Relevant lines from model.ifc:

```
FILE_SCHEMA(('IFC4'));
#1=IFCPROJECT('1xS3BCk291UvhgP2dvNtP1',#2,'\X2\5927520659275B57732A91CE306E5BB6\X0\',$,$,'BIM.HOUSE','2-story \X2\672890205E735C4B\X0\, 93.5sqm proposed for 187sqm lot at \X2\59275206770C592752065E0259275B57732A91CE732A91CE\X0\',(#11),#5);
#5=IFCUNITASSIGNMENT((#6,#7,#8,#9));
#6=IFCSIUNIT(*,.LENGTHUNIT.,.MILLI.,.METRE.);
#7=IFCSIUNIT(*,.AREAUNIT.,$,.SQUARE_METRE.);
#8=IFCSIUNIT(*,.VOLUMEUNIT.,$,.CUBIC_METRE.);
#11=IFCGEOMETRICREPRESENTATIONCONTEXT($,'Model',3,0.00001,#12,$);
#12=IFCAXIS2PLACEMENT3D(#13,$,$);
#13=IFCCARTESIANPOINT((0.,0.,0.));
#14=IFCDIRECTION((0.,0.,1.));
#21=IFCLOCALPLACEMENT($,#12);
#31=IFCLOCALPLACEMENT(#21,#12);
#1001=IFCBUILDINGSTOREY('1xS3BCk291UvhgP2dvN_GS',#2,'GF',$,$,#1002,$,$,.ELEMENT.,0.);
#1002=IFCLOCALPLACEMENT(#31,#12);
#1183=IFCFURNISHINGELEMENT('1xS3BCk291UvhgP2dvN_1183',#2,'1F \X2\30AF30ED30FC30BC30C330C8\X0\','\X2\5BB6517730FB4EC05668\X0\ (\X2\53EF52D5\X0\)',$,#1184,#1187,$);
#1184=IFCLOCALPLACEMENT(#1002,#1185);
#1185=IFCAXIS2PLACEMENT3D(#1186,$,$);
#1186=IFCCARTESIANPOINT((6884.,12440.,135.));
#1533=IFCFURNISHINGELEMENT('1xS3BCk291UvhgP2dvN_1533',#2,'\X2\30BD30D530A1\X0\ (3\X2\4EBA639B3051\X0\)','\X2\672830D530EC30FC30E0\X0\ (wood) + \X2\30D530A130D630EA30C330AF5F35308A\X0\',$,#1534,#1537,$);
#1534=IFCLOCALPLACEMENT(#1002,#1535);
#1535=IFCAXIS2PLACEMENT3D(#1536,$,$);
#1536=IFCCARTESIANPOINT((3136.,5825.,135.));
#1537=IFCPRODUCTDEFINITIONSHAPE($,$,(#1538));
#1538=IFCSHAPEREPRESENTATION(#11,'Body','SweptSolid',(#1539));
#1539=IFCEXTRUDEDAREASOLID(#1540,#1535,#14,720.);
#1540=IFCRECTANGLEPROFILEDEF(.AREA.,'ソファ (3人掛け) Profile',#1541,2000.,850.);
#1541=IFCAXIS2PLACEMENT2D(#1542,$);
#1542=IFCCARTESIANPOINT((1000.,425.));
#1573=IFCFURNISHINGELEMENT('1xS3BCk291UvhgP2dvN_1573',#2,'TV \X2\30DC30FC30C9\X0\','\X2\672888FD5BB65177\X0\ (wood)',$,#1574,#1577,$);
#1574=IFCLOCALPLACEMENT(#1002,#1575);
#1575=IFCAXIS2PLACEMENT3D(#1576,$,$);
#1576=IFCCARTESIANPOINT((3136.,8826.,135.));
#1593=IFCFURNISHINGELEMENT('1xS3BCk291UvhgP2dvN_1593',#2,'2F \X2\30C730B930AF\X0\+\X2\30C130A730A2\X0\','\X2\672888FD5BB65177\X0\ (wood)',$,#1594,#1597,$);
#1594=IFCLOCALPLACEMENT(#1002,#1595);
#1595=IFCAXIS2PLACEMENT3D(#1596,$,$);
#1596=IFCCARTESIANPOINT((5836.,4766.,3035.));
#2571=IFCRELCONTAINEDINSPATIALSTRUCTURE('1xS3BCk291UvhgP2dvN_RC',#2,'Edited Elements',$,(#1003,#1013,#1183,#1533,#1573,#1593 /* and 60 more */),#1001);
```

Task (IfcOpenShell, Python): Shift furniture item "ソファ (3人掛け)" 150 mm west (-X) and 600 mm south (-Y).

```python
import ifcopenshell
import ifcopenshell.api.geometry
import ifcopenshell.util.placement

model = ifcopenshell.open("model.ifc")

item = model.by_id(1533)
matrix = ifcopenshell.util.placement.get_local_placement(item.ObjectPlacement)
matrix[0, 3] -= 150.0
matrix[1, 3] -= 600.0
ifcopenshell.api.geometry.edit_object_placement(model, product=item, matrix=matrix, is_si=False)

print(ifcopenshell.util.placement.get_local_placement(item.ObjectPlacement).round(3) + 0.0)

model.write("model_updated.ifc")
```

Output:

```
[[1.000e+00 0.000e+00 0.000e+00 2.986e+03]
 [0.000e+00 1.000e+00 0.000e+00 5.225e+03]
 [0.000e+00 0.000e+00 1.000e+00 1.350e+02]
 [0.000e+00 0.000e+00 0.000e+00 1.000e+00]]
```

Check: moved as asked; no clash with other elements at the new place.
